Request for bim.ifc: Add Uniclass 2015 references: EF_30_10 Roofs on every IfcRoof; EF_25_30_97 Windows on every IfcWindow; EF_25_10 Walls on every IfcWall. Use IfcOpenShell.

First a look at what the model holds.

```python
import ifcopenshell

model = ifcopenshell.open("bim.ifc")
print(model.schema)
print("classifications:", [c.Name for c in model.by_type("IfcClassification")])
for ifc_class in ("IfcDoor", "IfcRoof", "IfcStair", "IfcWall", "IfcWindow"):
    print(ifc_class, len(model.by_type(ifc_class)))
```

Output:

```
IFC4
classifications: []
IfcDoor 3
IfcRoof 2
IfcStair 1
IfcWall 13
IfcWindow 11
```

```python
import ifcopenshell
import ifcopenshell.api.classification

model = ifcopenshell.open("bim.ifc")

system = ifcopenshell.api.classification.add_classification(model, classification="Uniclass 2015")

codes = {
    "IfcRoof": ("EF_30_10", "Roofs"),
    "IfcWindow": ("EF_25_30_97", "Windows"),
    "IfcWall": ("EF_25_10", "Walls"),
}
for ifc_class, (code, name) in codes.items():
    products = model.by_type(ifc_class)
    ifcopenshell.api.classification.add_reference(
        model, products=products, classification=system, identification=code, name=name
    )
    print(code, len(products))

model.write("bim_rev.ifc")
```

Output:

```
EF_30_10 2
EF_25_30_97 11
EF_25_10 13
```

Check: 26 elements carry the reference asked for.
